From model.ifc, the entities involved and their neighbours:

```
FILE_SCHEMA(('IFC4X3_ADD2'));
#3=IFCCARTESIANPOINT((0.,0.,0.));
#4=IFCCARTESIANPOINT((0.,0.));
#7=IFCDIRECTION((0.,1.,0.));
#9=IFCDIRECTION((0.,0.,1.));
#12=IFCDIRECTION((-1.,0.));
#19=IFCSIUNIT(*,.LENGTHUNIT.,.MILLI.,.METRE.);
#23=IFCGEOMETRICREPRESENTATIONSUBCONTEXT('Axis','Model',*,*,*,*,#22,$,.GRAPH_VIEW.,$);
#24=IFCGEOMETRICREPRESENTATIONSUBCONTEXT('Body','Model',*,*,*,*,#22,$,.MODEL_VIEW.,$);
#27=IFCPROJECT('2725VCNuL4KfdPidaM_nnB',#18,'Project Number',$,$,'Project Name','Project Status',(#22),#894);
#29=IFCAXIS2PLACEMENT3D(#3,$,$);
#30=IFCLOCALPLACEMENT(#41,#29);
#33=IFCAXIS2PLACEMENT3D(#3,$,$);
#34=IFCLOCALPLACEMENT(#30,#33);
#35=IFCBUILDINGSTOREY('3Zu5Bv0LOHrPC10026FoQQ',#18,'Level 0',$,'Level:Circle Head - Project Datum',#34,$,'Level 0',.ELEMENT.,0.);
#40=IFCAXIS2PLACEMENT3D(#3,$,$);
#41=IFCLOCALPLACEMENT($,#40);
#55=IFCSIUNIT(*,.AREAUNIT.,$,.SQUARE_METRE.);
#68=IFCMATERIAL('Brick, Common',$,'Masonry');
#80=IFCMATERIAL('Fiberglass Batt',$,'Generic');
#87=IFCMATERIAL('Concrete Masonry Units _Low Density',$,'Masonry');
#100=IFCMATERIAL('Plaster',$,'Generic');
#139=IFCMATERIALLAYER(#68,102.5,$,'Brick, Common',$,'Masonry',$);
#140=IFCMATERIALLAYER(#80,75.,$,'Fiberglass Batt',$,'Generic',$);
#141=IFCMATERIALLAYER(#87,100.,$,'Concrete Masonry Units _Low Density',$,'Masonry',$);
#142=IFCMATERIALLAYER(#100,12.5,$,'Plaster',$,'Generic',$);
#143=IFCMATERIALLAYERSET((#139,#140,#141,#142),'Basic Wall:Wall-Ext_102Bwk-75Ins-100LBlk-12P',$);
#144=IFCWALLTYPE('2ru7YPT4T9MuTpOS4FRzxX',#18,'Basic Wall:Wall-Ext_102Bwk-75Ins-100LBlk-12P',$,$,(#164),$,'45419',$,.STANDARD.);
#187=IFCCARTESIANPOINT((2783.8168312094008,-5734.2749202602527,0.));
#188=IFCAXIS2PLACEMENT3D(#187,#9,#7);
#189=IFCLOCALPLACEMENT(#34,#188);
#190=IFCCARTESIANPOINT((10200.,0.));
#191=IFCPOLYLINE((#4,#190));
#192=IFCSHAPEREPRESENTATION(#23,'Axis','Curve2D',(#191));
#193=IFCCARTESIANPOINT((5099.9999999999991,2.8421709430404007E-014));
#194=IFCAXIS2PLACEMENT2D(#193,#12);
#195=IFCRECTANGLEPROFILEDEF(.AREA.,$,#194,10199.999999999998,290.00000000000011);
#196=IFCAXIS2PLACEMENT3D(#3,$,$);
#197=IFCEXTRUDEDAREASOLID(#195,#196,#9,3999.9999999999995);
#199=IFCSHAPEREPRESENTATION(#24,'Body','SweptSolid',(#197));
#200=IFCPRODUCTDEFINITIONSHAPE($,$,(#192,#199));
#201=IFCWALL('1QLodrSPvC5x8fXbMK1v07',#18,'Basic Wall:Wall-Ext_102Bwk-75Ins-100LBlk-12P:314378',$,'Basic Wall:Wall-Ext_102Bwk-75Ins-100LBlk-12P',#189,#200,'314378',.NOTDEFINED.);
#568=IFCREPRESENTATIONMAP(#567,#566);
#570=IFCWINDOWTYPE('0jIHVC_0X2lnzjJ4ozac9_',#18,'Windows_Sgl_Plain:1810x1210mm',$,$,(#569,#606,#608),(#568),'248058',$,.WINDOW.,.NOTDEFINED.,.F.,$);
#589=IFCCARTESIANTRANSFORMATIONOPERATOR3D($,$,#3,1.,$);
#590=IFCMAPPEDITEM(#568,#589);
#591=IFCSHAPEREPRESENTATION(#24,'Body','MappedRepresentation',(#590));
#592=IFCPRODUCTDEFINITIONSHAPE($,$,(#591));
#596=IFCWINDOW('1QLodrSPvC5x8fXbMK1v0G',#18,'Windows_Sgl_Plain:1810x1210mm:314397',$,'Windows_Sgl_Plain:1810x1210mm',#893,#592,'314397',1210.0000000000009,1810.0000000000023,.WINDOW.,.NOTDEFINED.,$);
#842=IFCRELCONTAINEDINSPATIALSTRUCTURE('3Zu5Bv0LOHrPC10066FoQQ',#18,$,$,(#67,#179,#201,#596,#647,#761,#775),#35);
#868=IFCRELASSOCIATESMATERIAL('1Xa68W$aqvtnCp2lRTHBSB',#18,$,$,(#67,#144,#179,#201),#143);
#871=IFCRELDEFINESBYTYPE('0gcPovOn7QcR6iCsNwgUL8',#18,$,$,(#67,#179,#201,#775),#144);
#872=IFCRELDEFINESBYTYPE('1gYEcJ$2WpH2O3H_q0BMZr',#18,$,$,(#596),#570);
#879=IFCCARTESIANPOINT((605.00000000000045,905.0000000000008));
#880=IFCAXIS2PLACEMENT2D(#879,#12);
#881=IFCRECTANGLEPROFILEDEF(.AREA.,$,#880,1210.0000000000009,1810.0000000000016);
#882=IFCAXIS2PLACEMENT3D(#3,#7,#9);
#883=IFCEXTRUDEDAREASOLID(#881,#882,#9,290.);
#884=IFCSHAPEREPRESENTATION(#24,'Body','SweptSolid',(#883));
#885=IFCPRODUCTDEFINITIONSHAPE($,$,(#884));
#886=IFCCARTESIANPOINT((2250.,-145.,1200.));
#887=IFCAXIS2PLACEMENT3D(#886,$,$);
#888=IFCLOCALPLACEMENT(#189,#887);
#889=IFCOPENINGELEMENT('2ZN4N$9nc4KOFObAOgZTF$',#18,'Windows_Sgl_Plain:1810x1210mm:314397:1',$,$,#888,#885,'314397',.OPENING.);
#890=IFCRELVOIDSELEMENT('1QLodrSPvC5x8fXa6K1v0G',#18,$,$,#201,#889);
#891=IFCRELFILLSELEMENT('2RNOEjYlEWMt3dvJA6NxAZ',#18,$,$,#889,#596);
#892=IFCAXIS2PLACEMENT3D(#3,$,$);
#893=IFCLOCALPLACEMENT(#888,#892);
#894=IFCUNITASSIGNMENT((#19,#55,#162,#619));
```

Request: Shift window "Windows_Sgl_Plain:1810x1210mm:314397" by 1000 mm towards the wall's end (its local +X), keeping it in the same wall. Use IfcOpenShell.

```python
import ifcopenshell
import ifcopenshell.api.geometry
import ifcopenshell.util.placement
import ifcopenshell.util.unit

model = ifcopenshell.open("model.ifc")
unit_scale = ifcopenshell.util.unit.calculate_unit_scale(model)

window = model.by_guid("1QLodrSPvC5x8fXbMK1v0G")
opening = window.FillsVoids[0].RelatingOpeningElement
wall = opening.VoidsElements[0].RelatingBuildingElement

wall_matrix = ifcopenshell.util.placement.get_local_placement(wall.ObjectPlacement)
shift = wall_matrix[:3, 0] * 1 / unit_scale
before = ifcopenshell.util.placement.get_local_placement(window.ObjectPlacement)[:3, 3].copy()

# The window is placed relative to its opening, so it follows when the opening moves.
matrix = ifcopenshell.util.placement.get_local_placement(opening.ObjectPlacement)
matrix[:3, 3] += shift
ifcopenshell.api.geometry.edit_object_placement(
    model, product=opening, matrix=matrix, is_si=False, should_transform_children=True
)

after = ifcopenshell.util.placement.get_local_placement(window.ObjectPlacement)[:3, 3]
print("window moved by", (after - before).round(3) + 0.0)

model.write("model_edited.ifc")
```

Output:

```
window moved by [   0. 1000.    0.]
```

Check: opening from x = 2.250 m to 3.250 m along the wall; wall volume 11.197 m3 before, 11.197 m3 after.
